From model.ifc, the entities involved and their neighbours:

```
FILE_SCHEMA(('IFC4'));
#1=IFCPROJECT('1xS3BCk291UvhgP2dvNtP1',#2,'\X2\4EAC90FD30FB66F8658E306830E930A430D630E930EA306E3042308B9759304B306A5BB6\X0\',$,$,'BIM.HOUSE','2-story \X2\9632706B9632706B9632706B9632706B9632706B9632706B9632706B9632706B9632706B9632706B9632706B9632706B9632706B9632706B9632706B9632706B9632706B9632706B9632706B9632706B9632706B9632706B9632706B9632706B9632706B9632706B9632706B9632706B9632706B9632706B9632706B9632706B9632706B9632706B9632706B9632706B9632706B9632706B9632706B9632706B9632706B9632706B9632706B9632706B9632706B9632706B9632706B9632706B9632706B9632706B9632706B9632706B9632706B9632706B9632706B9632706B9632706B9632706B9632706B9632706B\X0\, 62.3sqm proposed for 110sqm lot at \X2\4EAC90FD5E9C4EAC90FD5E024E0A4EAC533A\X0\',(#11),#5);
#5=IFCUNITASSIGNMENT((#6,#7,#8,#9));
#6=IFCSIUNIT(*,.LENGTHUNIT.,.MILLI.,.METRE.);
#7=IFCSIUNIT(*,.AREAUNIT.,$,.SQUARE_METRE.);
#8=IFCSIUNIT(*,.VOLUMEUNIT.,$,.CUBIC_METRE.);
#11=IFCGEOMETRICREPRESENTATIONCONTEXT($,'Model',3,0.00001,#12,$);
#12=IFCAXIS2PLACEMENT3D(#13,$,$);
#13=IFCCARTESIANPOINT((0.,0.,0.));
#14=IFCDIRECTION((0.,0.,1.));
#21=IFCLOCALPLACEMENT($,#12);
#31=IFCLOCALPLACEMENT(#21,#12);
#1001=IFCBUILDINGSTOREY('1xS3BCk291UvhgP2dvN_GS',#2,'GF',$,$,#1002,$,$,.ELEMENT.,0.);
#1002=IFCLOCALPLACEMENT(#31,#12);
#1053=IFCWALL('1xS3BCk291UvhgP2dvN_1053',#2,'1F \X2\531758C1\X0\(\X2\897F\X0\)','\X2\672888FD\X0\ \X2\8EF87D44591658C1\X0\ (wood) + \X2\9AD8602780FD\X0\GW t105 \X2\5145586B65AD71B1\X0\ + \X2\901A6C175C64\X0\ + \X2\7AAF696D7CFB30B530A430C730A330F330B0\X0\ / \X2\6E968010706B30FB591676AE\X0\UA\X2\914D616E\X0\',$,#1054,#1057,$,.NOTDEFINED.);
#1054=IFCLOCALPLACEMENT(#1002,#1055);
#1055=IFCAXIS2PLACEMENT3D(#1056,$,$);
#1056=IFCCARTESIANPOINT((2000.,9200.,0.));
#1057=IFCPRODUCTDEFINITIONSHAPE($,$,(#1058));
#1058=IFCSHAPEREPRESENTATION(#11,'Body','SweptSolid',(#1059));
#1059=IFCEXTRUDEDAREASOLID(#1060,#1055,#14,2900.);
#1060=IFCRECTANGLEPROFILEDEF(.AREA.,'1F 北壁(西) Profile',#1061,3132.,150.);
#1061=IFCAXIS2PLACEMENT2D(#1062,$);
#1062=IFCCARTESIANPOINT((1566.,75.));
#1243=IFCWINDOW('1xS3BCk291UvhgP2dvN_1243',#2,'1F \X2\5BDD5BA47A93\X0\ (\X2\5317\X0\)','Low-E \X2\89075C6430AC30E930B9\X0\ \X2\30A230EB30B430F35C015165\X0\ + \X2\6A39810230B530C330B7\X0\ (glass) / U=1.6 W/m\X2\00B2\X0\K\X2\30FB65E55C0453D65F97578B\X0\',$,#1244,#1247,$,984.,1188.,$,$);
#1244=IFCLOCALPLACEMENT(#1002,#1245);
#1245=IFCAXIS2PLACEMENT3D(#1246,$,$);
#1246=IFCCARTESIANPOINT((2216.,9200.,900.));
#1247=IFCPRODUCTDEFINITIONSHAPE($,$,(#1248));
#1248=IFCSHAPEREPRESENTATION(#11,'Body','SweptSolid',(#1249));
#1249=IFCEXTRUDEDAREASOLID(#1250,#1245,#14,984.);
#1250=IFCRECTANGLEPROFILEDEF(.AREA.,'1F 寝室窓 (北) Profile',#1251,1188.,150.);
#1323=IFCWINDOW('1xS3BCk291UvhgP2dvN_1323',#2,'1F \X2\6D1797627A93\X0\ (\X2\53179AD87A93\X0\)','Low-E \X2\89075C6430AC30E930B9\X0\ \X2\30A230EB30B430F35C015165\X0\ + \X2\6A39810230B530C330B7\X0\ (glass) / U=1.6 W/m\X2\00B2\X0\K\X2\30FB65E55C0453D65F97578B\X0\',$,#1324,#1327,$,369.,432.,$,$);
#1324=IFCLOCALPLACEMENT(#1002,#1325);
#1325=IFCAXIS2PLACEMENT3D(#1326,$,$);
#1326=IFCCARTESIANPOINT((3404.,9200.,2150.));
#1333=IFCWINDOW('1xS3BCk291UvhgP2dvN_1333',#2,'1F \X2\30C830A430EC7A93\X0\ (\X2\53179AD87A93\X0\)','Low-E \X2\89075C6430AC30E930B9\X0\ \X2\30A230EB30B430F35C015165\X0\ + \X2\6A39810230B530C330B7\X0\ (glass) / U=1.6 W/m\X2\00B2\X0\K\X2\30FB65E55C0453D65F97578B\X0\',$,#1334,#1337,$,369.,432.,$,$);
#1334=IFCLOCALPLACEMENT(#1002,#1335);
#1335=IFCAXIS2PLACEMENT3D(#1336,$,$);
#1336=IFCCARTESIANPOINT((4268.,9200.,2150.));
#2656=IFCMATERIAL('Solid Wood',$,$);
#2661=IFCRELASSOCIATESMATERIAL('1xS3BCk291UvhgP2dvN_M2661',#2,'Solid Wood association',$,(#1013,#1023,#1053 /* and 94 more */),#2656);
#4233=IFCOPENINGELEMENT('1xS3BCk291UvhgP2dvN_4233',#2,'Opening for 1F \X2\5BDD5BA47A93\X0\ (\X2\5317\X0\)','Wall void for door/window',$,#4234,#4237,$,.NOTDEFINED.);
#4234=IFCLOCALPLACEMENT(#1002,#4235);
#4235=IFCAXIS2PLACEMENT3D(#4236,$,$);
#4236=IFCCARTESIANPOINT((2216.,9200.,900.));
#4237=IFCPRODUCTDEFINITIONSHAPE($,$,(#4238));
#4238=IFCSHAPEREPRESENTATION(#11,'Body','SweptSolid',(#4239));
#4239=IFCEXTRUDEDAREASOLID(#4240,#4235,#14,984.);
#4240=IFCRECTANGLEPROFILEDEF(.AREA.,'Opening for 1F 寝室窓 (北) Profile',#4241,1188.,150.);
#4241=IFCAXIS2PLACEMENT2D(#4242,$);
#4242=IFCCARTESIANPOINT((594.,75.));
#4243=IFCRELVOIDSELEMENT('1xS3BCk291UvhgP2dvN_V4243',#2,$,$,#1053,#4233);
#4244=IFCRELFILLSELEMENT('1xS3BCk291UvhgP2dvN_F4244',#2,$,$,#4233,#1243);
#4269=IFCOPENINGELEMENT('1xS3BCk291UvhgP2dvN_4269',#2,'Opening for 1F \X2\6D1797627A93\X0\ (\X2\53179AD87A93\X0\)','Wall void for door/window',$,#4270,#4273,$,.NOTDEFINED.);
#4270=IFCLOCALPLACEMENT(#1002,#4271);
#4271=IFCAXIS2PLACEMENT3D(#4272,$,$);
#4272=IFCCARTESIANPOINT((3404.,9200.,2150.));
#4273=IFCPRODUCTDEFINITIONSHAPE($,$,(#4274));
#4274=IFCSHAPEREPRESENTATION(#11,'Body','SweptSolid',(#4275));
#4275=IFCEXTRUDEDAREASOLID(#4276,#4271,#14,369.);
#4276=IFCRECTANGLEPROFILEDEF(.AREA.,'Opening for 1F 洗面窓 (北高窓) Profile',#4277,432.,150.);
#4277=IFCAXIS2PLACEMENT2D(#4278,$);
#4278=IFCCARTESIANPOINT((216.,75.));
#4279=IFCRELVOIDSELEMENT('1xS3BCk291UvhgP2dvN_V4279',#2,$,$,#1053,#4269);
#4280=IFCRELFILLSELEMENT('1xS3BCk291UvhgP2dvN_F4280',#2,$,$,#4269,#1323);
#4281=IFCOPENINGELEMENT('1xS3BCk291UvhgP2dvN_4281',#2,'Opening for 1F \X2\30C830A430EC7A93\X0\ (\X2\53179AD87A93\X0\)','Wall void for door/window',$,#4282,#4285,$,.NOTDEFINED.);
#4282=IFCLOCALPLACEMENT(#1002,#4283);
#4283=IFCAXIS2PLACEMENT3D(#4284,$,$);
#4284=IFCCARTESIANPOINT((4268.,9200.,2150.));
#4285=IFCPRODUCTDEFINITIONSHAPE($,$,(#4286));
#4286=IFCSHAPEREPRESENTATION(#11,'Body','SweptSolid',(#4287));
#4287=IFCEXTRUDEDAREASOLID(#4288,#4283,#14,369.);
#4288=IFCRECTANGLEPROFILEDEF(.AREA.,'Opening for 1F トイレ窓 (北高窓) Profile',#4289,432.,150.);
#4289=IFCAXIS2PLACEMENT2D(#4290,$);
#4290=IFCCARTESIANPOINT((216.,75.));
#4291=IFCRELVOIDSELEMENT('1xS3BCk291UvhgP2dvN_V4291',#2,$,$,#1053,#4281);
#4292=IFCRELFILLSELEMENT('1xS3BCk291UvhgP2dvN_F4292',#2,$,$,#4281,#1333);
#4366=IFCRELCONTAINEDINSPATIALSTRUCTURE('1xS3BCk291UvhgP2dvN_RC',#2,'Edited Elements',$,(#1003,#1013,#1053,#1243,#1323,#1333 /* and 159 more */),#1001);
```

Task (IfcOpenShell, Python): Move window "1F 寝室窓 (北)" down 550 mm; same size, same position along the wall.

```python
import numpy as np
import ifcopenshell
import ifcopenshell.api.geometry
import ifcopenshell.util.placement
import ifcopenshell.util.unit

model = ifcopenshell.open("model.ifc")
unit_scale = ifcopenshell.util.unit.calculate_unit_scale(model)

window = model.by_id(1243)
opening = window.FillsVoids[0].RelatingOpeningElement
dz = -550.0

shift = np.array([0.0, 0.0, dz])
# The window is not placed relative to its opening, so move both.
for product in (opening, window):
    matrix = ifcopenshell.util.placement.get_local_placement(product.ObjectPlacement)
    matrix[:3, 3] += shift
    ifcopenshell.api.geometry.edit_object_placement(model, product=product, matrix=matrix, is_si=False)

print(f"moved by {dz * unit_scale:+.3f} m")

model.write("model_updated.ifc")
```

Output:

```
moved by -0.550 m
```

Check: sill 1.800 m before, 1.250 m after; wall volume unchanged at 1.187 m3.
